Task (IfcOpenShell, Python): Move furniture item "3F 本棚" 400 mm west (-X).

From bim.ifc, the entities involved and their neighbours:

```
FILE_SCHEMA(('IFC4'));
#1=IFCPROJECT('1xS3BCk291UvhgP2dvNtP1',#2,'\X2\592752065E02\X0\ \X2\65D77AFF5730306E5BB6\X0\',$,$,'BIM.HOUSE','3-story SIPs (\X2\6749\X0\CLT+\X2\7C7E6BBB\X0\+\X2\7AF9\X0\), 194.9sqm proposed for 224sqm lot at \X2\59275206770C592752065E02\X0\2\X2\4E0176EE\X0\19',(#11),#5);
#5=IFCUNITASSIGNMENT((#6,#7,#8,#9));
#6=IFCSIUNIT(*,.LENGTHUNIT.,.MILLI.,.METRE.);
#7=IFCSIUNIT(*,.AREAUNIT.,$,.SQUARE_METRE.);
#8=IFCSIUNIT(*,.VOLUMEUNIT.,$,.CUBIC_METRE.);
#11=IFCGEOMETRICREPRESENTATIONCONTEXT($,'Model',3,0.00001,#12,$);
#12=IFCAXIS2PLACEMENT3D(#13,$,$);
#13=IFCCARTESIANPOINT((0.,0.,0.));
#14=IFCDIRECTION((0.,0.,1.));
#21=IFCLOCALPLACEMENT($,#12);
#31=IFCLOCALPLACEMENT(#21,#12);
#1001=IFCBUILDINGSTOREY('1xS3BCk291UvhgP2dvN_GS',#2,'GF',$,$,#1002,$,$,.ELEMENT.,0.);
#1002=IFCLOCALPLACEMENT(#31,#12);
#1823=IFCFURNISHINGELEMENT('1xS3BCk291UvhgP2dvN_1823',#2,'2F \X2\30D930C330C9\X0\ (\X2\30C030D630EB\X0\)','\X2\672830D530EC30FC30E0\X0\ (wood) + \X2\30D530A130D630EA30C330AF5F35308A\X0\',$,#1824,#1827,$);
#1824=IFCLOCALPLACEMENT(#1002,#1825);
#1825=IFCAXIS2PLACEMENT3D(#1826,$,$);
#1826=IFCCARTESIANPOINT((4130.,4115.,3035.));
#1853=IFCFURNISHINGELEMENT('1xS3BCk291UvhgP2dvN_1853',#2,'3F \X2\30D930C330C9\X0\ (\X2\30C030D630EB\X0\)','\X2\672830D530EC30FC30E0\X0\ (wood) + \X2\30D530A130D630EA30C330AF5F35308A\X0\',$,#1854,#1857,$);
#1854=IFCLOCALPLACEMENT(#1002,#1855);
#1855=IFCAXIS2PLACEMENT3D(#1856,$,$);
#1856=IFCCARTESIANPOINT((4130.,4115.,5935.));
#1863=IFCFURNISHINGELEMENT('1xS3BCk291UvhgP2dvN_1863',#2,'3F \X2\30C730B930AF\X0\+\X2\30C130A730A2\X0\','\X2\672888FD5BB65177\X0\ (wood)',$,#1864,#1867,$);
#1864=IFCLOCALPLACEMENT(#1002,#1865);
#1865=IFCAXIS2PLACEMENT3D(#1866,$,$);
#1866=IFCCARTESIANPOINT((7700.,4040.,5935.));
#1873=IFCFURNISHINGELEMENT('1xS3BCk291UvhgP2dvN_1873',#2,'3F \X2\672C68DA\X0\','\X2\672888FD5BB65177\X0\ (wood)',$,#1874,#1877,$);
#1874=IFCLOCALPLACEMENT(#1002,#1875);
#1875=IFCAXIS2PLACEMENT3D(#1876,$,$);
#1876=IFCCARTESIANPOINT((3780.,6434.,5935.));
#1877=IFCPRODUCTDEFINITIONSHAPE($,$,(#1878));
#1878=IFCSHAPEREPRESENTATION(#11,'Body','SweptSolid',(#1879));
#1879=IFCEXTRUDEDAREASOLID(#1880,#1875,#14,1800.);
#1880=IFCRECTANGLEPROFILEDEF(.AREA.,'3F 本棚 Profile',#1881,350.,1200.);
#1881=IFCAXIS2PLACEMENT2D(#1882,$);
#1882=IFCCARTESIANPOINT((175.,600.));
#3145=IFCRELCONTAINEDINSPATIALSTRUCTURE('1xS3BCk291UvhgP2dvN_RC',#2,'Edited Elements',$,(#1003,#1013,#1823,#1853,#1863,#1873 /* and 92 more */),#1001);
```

```python
import ifcopenshell
import ifcopenshell.api.geometry
import ifcopenshell.util.placement
import ifcopenshell.util.unit

model = ifcopenshell.open("bim.ifc")
unit_scale = ifcopenshell.util.unit.calculate_unit_scale(model)

item = model.by_id(1873)
matrix = ifcopenshell.util.placement.get_local_placement(item.ObjectPlacement)
matrix[0, 3] -= 0.4 / unit_scale
ifcopenshell.api.geometry.edit_object_placement(model, product=item, matrix=matrix, is_si=False)

print(ifcopenshell.util.placement.get_local_placement(item.ObjectPlacement).round(3) + 0.0)

model.write("bim_updated.ifc")
```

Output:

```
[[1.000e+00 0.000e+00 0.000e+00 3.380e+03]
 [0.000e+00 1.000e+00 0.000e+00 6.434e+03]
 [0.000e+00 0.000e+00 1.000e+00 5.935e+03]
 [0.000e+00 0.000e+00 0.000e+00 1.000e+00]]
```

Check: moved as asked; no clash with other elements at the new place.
